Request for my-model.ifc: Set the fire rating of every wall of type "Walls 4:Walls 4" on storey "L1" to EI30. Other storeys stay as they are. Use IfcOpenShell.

First a look at what the model holds.

```python
import ifcopenshell
import ifcopenshell.util.element

model = ifcopenshell.open("my-model.ifc")
print(model.schema)
storey = next(s for s in model.by_type("IfcBuildingStorey") if s.Name == "L1")
walls = [e for e in ifcopenshell.util.element.get_decomposition(storey) if e.is_a("IfcWall")]
seen = {}
for e in walls:
    element_type = ifcopenshell.util.element.get_type(e)
    key = (element_type.Name if element_type != e and element_type else None, ifcopenshell.util.element.get_pset(e, "Pset_WallCommon", "FireRating"))
    seen[key] = seen.get(key, 0) + 1
for (name, value), count in sorted(seen.items(), key=str):
    print(count, "x", name, "|", value)
```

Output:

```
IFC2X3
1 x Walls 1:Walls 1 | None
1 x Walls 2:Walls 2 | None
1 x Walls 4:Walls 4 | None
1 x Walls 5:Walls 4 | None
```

```python
import ifcopenshell
import ifcopenshell.api.pset
import ifcopenshell.util.element

model = ifcopenshell.open("my-model.ifc")

storey = next(s for s in model.by_type("IfcBuildingStorey") if s.Name == "L1")
walls = [e for e in ifcopenshell.util.element.get_decomposition(storey) if e.is_a("IfcWall")]

count = 0
for e in walls:
    element_type = ifcopenshell.util.element.get_type(e)
    if element_type in (None, e) or element_type.Name != "Walls 4:Walls 4":
        continue
    # add_pset returns the element's existing set when there is one.
    pset = ifcopenshell.api.pset.add_pset(model, product=e, name="Pset_WallCommon")
    ifcopenshell.api.pset.edit_pset(model, pset=pset, properties={"FireRating": "EI30"})
    count += 1

print(count, "walls updated")

model.write("my-model_updated.ifc")
```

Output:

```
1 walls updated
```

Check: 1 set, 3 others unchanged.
